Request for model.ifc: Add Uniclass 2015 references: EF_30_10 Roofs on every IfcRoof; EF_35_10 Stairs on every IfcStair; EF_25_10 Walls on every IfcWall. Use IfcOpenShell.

First a look at what the model holds.

```python
import ifcopenshell

model = ifcopenshell.open("model.ifc")
print(model.schema)
print("classifications:", [c.Name for c in model.by_type("IfcClassification")])
for ifc_class in ("IfcDoor", "IfcRoof", "IfcStair", "IfcWall", "IfcWindow"):
    print(ifc_class, len(model.by_type(ifc_class)))
```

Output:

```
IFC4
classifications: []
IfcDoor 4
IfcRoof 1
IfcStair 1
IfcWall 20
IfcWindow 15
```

```python
import ifcopenshell
import ifcopenshell.api.classification

model = ifcopenshell.open("model.ifc")

system = ifcopenshell.api.classification.add_classification(model, classification="Uniclass 2015")

codes = {
    "IfcRoof": ("EF_30_10", "Roofs"),
    "IfcStair": ("EF_35_10", "Stairs"),
    "IfcWall": ("EF_25_10", "Walls"),
}
for ifc_class, (code, name) in codes.items():
    products = model.by_type(ifc_class)
    ifcopenshell.api.classification.add_reference(
        model, products=products, classification=system, identification=code, name=name
    )
    print(code, len(products))

model.write("model_rev.ifc")
```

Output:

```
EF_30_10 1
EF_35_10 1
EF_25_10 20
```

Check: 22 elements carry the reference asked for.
